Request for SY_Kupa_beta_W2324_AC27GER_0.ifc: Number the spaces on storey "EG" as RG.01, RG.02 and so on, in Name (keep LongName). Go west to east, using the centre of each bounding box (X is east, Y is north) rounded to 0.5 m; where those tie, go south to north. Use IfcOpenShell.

First a look at what the model holds.

```python
import ifcopenshell
import ifcopenshell.util.element
import ifcopenshell.util.placement

model = ifcopenshell.open("SY_Kupa_beta_W2324_AC27GER_0.ifc")
print(model.schema)
storey = next(s for s in model.by_type("IfcBuildingStorey") if s.Name == "EG")
spaces = [e for e in ifcopenshell.util.element.get_decomposition(storey) if e.is_a("IfcSpace")]
for e in sorted(spaces, key=lambda e: e.id()):
    origin = ifcopenshell.util.placement.get_local_placement(e.ObjectPlacement)[:3, 3]
    print(e.id(), e.Name, e.LongName, origin.round(2) + 0.0, sep=" | ")
```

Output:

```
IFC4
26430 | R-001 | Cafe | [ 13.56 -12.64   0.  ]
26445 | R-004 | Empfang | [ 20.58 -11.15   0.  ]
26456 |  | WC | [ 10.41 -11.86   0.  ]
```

```python
import ifcopenshell
import ifcopenshell.geom
import ifcopenshell.util.element
import ifcopenshell.util.shape

model = ifcopenshell.open("SY_Kupa_beta_W2324_AC27GER_0.ifc")
settings = ifcopenshell.geom.settings()
settings.set("use-world-coords", True)


def centre(element):
    shape = ifcopenshell.geom.create_shape(settings, element)
    return ifcopenshell.util.shape.get_bbox_centroid(shape.geometry)


storey = next(s for s in model.by_type("IfcBuildingStorey") if s.Name == "EG")
spaces = [e for e in ifcopenshell.util.element.get_decomposition(storey) if e.is_a("IfcSpace")]

# Insertion points can sit at a corner or the storey origin, so sort by the geometry (in metres).
centres = {e: centre(e) for e in spaces}
spaces.sort(key=lambda e: (round(centres[e][0] / 0.5), centres[e][1]))

for i, e in enumerate(spaces, start=1):
    number = f"RG.{i:02d}"
    e.Name = number
    print(e.id(), number)

model.write("SY_Kupa_beta_W2324_AC27GER_0_rev.ifc")
```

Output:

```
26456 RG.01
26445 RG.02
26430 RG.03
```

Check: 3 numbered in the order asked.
